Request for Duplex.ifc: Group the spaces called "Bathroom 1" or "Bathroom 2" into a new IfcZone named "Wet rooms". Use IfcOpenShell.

First a look at what the model holds.

```python
import ifcopenshell

model = ifcopenshell.open("Duplex.ifc")
print(model.schema)
seen = {}
for space in model.by_type("IfcSpace"):
    seen[space.LongName] = seen.get(space.LongName, 0) + 1
for name, count in sorted(seen.items(), key=str):
    print(count, "x", name)
print("zones:", [z.Name for z in model.by_type("IfcZone")][:20])
```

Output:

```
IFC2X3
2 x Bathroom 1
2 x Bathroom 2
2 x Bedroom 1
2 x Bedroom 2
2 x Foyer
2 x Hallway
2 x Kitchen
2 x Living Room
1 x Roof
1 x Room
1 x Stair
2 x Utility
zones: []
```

```python
import ifcopenshell
import ifcopenshell.api.group
import ifcopenshell.api.root

model = ifcopenshell.open("Duplex.ifc")

names = {"Bathroom 1", "Bathroom 2"}
spaces = [s for s in model.by_type("IfcSpace") if s.LongName in names]

zone = ifcopenshell.api.root.create_entity(model, ifc_class="IfcZone", name="Wet rooms")
ifcopenshell.api.group.assign_group(model, products=spaces, group=zone)
print(len(spaces), "spaces in", zone.Name)

model.write("Duplex_edited.ifc")
```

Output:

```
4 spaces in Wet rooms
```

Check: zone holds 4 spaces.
